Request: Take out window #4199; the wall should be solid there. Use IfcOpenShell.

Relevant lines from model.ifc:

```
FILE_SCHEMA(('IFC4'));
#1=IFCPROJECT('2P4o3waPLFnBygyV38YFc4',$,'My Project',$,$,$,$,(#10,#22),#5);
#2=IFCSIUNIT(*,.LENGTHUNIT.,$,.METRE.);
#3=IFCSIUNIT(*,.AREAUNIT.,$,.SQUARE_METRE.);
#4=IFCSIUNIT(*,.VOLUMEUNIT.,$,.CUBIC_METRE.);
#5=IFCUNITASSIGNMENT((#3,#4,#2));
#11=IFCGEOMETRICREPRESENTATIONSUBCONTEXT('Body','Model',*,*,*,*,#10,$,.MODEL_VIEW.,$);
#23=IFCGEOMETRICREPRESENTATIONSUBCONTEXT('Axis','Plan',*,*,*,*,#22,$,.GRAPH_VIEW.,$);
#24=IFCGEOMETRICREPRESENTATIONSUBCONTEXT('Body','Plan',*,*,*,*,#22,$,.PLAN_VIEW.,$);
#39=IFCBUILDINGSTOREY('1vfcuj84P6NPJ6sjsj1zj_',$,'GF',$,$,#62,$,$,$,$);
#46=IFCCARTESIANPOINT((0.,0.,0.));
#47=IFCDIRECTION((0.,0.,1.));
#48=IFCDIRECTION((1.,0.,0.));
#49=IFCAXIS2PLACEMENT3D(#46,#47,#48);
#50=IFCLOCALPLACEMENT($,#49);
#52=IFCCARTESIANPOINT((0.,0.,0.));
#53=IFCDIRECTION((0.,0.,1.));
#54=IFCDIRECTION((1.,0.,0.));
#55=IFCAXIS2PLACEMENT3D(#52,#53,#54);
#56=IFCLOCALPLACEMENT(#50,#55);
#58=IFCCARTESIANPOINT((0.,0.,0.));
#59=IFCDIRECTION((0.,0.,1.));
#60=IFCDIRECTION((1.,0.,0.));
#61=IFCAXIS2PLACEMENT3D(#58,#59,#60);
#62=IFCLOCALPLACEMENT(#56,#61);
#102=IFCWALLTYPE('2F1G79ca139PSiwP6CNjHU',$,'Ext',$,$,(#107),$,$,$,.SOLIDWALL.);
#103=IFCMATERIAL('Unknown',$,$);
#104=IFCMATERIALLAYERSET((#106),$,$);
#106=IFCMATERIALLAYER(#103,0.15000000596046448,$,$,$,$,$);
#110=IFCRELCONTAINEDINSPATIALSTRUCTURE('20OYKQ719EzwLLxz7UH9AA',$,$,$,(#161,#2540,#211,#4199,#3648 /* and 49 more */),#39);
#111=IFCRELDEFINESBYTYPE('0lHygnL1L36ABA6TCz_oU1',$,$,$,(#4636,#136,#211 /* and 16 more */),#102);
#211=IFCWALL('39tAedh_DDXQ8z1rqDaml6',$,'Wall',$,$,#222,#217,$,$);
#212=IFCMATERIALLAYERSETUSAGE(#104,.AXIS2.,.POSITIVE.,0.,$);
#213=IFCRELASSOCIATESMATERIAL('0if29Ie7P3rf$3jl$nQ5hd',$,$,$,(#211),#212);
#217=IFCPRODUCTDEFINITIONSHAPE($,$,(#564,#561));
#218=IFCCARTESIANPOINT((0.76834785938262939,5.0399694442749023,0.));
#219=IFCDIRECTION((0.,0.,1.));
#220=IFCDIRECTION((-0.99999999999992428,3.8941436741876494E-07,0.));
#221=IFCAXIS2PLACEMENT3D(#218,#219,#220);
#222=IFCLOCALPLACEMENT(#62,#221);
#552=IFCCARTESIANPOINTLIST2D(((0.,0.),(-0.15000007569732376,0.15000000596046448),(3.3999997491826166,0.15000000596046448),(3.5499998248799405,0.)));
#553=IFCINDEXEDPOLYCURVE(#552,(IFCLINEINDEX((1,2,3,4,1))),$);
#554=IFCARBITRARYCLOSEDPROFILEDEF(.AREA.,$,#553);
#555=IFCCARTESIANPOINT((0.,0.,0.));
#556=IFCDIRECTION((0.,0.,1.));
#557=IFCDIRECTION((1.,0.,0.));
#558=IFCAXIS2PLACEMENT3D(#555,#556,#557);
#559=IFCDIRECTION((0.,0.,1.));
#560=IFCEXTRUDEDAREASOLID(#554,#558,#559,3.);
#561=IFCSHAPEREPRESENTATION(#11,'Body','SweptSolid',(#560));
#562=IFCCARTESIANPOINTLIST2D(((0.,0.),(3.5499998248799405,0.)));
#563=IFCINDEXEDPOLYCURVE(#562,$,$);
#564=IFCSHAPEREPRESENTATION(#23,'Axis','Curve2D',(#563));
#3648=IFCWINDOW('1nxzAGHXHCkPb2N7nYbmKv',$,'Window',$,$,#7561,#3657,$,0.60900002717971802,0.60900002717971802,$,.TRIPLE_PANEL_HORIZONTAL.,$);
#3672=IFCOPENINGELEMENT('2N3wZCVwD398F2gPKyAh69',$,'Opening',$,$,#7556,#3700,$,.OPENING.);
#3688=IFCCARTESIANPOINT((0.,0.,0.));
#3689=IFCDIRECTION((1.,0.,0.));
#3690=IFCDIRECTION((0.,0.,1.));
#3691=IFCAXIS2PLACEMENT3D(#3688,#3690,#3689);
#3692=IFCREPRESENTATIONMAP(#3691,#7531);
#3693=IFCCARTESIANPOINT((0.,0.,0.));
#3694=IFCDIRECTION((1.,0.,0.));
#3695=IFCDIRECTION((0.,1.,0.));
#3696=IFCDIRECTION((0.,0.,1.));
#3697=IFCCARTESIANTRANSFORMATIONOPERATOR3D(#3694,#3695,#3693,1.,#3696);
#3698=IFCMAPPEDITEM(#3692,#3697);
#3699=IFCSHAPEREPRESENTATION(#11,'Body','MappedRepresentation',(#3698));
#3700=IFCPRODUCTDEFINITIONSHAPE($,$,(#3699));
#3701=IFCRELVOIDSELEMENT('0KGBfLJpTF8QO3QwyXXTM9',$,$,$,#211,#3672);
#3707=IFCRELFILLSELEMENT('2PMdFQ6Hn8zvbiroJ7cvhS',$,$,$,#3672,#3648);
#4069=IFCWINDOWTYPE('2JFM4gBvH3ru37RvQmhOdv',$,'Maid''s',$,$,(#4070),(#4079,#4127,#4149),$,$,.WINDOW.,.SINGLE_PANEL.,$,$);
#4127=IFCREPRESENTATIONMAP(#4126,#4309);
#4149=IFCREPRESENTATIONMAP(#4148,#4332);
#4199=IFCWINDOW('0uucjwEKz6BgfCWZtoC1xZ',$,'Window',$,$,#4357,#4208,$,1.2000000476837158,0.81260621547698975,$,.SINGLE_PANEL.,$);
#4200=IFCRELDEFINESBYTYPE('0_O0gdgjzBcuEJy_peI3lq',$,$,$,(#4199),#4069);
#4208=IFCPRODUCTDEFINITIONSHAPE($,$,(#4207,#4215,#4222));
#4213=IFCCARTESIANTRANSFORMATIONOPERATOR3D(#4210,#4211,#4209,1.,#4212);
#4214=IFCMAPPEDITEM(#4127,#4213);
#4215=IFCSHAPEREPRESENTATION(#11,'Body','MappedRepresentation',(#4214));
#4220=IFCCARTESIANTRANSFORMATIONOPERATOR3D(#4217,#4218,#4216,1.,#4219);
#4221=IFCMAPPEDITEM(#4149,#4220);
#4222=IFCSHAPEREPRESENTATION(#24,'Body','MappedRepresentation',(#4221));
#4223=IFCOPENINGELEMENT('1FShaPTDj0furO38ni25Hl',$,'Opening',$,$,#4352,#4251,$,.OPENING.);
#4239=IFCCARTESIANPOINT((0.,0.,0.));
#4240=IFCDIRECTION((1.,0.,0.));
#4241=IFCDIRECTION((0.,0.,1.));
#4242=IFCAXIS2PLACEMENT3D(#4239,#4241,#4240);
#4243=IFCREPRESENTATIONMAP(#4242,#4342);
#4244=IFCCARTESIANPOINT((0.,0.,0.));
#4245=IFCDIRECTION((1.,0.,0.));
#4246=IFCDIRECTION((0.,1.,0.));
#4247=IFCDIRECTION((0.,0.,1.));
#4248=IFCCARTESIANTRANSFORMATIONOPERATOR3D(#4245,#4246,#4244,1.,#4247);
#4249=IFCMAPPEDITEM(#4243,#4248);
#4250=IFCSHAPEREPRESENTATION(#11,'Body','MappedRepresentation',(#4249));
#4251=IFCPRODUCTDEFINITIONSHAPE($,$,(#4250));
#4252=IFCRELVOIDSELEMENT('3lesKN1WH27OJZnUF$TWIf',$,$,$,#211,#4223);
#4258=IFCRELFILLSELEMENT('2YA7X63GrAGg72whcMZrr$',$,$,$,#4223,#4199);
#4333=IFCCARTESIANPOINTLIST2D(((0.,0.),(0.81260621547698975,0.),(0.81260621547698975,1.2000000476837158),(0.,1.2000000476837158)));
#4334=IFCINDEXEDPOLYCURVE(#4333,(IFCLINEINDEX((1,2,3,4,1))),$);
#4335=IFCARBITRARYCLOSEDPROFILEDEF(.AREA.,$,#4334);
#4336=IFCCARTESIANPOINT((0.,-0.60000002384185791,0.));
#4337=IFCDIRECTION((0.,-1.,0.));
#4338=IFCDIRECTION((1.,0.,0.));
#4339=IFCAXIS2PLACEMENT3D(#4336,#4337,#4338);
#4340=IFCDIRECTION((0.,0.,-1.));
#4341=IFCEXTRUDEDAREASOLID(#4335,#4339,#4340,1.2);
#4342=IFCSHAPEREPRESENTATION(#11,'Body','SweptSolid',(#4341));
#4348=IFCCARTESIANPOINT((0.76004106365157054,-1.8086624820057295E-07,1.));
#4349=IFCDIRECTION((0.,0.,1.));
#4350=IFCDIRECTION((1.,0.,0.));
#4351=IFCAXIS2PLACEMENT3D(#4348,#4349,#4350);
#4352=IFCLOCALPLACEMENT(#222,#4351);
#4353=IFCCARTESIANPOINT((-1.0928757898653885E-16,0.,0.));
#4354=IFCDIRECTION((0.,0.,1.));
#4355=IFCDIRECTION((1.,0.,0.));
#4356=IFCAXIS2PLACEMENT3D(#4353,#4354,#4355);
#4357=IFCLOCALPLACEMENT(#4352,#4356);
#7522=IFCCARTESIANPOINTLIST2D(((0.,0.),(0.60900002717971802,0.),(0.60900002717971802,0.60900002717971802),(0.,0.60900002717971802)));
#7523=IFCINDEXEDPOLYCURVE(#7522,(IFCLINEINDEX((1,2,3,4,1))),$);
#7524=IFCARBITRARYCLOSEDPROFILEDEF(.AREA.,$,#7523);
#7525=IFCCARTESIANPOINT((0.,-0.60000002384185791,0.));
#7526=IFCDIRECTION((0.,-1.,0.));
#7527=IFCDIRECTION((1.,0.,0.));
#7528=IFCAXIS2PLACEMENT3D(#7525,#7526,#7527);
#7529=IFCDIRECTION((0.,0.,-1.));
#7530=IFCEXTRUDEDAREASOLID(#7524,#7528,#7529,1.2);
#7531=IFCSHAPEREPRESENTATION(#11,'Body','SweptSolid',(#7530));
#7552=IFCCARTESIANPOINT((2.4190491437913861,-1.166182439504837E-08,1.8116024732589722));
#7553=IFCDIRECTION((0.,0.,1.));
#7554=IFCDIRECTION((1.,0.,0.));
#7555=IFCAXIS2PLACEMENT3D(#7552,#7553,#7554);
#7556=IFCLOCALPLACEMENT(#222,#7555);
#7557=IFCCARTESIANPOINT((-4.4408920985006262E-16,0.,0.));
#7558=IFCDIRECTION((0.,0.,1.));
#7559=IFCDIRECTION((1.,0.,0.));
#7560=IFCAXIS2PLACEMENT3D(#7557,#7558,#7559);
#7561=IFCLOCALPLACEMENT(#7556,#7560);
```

```python
import ifcopenshell
import ifcopenshell.api.feature
import ifcopenshell.api.root
import ifcopenshell.geom
import ifcopenshell.util.shape

model = ifcopenshell.open("model.ifc")
settings = ifcopenshell.geom.settings()


def volume(element):
    """Net volume in cubic metres, openings subtracted."""
    shape = ifcopenshell.geom.create_shape(settings, element)
    return ifcopenshell.util.shape.get_volume(shape.geometry)


window = model.by_guid("0uucjwEKz6BgfCWZtoC1xZ")
opening = window.FillsVoids[0].RelatingOpeningElement
wall = opening.VoidsElements[0].RelatingBuildingElement
before = volume(wall)

ifcopenshell.api.root.remove_product(model, product=window)
ifcopenshell.api.feature.remove_feature(model, feature=opening)

after = volume(wall)

print(f"wall volume {before:.3f} -> {after:.3f} m3")

model.write("model_edited.ifc")
```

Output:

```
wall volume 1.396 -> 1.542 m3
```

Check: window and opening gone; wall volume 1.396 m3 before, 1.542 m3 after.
